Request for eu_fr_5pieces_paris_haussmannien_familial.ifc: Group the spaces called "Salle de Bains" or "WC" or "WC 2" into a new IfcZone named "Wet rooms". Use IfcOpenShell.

First a look at what the model holds.

```python
import ifcopenshell

model = ifcopenshell.open("eu_fr_5pieces_paris_haussmannien_familial.ifc")
print(model.schema)
seen = {}
for space in model.by_type("IfcSpace"):
    seen[space.LongName] = seen.get(space.LongName, 0) + 1
for name, count in sorted(seen.items(), key=str):
    print(count, "x", name)
print("zones:", [z.Name for z in model.by_type("IfcZone")][:20])
```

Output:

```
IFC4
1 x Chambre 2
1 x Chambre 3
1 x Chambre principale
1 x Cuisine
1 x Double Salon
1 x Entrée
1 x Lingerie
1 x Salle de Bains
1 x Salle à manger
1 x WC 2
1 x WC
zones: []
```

```python
import ifcopenshell
import ifcopenshell.api.group
import ifcopenshell.api.root

model = ifcopenshell.open("eu_fr_5pieces_paris_haussmannien_familial.ifc")

names = {"Salle de Bains", "WC", "WC 2"}
spaces = [s for s in model.by_type("IfcSpace") if s.LongName in names]

zone = ifcopenshell.api.root.create_entity(model, ifc_class="IfcZone", name="Wet rooms")
ifcopenshell.api.group.assign_group(model, products=spaces, group=zone)
print(len(spaces), "spaces in", zone.Name)

model.write("eu_fr_5pieces_paris_haussmannien_familial_updated.ifc")
```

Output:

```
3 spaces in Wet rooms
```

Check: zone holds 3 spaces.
